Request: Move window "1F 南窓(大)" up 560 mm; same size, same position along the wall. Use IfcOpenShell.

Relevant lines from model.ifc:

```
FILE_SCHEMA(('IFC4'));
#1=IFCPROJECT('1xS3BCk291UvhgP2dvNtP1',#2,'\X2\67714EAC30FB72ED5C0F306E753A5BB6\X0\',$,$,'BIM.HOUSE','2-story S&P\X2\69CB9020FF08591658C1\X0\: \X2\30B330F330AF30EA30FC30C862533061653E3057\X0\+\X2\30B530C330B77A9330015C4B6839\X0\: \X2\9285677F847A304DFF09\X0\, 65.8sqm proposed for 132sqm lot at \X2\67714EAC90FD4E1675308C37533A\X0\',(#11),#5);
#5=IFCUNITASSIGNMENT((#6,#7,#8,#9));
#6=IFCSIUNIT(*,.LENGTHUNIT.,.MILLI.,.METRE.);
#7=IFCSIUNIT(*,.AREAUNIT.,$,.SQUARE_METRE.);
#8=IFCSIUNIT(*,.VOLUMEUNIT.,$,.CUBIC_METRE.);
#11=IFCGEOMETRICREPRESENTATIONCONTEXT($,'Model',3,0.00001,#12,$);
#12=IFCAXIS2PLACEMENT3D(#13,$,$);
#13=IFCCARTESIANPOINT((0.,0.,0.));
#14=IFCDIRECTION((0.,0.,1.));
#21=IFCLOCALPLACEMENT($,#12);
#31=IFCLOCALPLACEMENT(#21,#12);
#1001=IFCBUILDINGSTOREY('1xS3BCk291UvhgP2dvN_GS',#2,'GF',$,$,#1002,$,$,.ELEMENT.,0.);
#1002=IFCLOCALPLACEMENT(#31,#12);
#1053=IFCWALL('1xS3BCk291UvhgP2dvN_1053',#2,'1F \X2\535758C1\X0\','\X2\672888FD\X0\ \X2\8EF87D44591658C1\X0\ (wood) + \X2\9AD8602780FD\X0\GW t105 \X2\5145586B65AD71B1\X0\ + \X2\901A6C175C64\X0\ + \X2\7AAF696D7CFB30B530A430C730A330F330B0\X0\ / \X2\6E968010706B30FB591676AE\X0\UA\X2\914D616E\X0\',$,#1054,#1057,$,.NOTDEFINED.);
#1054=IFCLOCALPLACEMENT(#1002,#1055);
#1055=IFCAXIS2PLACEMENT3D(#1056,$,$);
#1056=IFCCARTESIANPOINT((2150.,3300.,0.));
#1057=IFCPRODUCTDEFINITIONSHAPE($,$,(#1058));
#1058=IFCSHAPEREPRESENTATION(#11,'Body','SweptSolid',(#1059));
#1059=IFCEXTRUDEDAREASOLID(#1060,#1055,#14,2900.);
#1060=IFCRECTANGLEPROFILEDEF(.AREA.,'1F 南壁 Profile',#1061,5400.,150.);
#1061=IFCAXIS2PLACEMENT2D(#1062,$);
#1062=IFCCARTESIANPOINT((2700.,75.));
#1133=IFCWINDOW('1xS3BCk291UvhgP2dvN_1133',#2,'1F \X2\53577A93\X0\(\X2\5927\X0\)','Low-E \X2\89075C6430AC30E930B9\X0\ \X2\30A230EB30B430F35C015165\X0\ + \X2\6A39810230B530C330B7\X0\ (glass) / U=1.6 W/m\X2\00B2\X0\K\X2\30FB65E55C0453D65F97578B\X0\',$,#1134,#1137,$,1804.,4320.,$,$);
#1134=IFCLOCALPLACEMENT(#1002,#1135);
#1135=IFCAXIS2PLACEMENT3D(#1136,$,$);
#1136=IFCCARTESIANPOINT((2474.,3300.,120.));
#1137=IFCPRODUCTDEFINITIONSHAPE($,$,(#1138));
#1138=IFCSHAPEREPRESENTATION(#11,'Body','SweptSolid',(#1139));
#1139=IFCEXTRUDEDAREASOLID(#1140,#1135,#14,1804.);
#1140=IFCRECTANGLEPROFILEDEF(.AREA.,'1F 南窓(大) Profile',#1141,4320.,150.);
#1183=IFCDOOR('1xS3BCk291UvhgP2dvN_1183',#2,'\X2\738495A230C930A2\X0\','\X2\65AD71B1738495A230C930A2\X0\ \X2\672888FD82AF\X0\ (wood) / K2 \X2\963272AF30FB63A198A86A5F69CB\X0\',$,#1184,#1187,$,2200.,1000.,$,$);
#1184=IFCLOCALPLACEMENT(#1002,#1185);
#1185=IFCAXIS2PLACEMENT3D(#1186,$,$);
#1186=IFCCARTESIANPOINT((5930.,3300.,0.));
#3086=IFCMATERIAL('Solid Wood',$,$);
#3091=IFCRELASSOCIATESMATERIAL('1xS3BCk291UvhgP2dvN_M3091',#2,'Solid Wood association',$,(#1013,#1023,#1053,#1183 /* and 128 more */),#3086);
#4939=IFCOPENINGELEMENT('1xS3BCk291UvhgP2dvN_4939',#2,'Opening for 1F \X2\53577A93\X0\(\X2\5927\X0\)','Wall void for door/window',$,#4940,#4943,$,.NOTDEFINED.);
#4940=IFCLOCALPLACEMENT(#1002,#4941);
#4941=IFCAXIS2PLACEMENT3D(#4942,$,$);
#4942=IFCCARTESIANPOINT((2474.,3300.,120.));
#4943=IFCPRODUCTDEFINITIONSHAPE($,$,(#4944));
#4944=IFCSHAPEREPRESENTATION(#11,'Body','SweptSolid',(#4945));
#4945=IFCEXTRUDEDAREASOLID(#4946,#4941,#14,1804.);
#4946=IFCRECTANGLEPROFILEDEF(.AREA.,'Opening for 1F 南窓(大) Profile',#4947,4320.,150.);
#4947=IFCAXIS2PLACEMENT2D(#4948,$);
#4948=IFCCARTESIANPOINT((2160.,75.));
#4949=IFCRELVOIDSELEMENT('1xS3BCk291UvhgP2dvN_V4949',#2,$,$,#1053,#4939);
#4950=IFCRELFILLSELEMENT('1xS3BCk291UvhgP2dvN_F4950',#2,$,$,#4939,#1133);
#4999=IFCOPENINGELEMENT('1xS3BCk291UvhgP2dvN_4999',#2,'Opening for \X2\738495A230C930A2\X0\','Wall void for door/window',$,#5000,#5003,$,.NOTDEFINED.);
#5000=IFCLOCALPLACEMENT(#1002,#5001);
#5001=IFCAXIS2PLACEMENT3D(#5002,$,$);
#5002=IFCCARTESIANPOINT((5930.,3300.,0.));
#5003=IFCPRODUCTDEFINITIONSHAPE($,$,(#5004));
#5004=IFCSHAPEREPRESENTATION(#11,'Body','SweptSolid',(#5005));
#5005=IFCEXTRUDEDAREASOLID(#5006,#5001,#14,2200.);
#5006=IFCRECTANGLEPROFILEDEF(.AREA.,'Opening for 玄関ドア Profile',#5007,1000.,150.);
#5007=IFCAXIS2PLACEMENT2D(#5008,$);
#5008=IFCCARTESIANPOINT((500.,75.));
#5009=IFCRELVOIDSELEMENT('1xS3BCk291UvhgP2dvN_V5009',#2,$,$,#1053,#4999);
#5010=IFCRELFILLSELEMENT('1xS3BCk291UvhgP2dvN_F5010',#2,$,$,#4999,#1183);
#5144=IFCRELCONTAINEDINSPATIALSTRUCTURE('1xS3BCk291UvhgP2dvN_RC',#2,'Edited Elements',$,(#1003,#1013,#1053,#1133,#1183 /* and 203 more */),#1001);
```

```python
import numpy as np
import ifcopenshell
import ifcopenshell.api.geometry
import ifcopenshell.util.placement
import ifcopenshell.util.unit

model = ifcopenshell.open("model.ifc")
unit_scale = ifcopenshell.util.unit.calculate_unit_scale(model)

window = model.by_guid("1xS3BCk291UvhgP2dvN_1133")
opening = window.FillsVoids[0].RelatingOpeningElement
dz = 560.0

shift = np.array([0.0, 0.0, dz])
# The window is not placed relative to its opening, so move both.
for product in (opening, window):
    matrix = ifcopenshell.util.placement.get_local_placement(product.ObjectPlacement)
    matrix[:3, 3] += shift
    ifcopenshell.api.geometry.edit_object_placement(model, product=product, matrix=matrix, is_si=False)

print(f"moved by {dz * unit_scale:+.3f} m")

model.write("model-out.ifc")
```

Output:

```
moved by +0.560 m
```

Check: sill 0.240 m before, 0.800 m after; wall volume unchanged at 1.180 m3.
